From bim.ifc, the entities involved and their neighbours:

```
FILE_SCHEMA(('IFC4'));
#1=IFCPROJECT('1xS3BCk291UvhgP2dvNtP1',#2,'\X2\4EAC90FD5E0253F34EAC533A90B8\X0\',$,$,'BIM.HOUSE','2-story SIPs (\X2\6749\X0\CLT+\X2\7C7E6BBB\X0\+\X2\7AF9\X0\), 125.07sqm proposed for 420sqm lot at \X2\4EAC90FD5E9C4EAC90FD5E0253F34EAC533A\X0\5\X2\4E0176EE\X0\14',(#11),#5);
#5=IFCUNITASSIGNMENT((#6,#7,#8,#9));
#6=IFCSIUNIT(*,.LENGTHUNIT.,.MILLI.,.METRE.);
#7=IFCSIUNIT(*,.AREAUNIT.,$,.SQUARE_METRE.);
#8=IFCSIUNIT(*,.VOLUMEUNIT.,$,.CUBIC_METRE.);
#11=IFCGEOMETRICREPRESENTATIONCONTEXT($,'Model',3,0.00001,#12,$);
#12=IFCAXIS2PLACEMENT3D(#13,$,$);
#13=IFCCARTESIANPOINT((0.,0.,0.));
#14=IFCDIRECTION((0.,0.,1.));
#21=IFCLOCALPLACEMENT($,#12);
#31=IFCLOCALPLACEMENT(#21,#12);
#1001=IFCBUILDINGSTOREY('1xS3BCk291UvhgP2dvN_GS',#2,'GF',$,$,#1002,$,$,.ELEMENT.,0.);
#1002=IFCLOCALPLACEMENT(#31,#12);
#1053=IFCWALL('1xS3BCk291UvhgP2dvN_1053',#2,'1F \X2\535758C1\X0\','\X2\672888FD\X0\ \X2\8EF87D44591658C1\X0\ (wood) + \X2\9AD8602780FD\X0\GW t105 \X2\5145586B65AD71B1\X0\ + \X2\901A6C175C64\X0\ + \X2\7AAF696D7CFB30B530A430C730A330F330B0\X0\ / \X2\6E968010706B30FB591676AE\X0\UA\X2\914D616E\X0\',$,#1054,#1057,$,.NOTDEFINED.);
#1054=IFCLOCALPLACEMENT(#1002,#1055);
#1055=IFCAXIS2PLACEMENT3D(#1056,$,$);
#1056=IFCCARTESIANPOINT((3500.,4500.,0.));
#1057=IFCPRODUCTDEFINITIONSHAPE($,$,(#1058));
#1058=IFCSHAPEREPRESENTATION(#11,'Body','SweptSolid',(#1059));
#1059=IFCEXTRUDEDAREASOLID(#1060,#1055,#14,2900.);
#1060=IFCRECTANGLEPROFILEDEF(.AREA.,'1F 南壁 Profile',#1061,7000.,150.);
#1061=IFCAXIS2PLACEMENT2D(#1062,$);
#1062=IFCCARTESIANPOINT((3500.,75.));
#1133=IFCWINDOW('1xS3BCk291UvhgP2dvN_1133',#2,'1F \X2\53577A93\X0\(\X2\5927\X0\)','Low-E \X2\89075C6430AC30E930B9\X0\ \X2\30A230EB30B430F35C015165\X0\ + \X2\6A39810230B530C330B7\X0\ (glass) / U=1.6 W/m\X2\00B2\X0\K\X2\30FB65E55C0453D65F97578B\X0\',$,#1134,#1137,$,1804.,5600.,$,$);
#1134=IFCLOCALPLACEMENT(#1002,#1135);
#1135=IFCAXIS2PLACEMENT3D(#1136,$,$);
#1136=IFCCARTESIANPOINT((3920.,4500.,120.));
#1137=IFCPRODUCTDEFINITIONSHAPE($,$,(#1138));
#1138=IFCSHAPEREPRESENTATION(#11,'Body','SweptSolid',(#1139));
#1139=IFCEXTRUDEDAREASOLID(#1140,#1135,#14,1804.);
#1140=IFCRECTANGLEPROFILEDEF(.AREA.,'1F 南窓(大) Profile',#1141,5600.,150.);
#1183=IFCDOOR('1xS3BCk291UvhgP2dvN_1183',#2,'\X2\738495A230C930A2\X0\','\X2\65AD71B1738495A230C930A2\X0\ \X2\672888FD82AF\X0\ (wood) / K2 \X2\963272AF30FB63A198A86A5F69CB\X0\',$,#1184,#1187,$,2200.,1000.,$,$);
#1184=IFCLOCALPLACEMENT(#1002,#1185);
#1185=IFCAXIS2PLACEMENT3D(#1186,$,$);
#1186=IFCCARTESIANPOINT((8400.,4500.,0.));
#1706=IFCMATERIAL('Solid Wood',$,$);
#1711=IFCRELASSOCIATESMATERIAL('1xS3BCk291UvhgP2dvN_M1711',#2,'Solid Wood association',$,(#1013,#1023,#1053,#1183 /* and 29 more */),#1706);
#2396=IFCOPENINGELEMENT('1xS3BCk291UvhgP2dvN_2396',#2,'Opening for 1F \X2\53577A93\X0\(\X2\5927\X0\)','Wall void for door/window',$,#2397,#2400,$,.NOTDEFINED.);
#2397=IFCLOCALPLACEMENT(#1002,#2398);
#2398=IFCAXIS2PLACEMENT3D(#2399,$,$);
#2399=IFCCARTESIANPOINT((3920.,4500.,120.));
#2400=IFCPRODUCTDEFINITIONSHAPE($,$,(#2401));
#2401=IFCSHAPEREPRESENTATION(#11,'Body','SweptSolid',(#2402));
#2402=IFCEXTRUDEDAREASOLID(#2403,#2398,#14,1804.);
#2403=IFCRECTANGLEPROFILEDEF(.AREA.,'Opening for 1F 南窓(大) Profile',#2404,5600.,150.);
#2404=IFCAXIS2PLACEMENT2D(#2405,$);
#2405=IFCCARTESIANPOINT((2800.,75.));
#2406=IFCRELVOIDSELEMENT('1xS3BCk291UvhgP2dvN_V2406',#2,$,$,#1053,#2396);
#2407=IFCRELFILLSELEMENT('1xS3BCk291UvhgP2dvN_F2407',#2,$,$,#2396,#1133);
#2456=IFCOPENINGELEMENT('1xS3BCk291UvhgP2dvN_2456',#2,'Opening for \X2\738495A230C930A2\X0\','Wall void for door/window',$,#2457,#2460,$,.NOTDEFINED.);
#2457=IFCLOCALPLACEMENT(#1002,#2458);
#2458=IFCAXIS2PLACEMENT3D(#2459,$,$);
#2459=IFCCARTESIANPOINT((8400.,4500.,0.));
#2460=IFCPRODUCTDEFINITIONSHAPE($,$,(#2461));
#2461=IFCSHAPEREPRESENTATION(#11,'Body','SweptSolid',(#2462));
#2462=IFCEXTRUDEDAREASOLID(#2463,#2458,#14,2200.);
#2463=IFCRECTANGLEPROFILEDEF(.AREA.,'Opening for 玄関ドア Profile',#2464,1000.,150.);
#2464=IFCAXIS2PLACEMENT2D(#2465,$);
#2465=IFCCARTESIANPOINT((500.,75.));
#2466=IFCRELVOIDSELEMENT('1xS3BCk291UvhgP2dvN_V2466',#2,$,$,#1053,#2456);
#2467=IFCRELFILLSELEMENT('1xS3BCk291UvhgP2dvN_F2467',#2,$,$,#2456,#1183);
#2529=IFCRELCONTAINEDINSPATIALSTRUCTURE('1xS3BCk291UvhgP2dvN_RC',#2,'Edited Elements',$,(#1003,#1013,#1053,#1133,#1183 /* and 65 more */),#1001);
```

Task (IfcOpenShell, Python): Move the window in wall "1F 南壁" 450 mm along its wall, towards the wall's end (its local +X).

```python
import ifcopenshell
import ifcopenshell.api.geometry
import ifcopenshell.util.placement

model = ifcopenshell.open("bim.ifc")

window = model.by_guid("1xS3BCk291UvhgP2dvN_1133")
opening = window.FillsVoids[0].RelatingOpeningElement
wall = opening.VoidsElements[0].RelatingBuildingElement

wall_matrix = ifcopenshell.util.placement.get_local_placement(wall.ObjectPlacement)
shift = wall_matrix[:3, 0] * 450.0
before = ifcopenshell.util.placement.get_local_placement(window.ObjectPlacement)[:3, 3].copy()

# The window is not placed relative to its opening, so move both.
for product in (opening, window):
    matrix = ifcopenshell.util.placement.get_local_placement(product.ObjectPlacement)
    matrix[:3, 3] += shift
    ifcopenshell.api.geometry.edit_object_placement(model, product=product, matrix=matrix, is_si=False)

after = ifcopenshell.util.placement.get_local_placement(window.ObjectPlacement)[:3, 3]
print("window moved by", (after - before).round(3) + 0.0)

model.write("bim_updated.ifc")
```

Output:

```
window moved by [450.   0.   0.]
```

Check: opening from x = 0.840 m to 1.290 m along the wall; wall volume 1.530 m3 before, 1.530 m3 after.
